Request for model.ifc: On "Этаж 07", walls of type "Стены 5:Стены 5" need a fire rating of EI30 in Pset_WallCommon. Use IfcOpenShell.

First a look at what the model holds.

```python
import ifcopenshell
import ifcopenshell.util.element

model = ifcopenshell.open("model.ifc")
print(model.schema)
storey = next(s for s in model.by_type("IfcBuildingStorey") if s.Name == "Этаж 07")
walls = [e for e in ifcopenshell.util.element.get_decomposition(storey) if e.is_a("IfcWall")]
seen = {}
for e in walls:
    element_type = ifcopenshell.util.element.get_type(e)
    key = (element_type.Name if element_type != e and element_type else None, ifcopenshell.util.element.get_pset(e, "Pset_WallCommon", "FireRating"))
    seen[key] = seen.get(key, 0) + 1
for (name, value), count in sorted(seen.items(), key=str):
    print(count, "x", name, "|", value)
```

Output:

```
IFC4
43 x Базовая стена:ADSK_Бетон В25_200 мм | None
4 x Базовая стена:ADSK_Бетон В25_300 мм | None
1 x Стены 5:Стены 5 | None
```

```python
import ifcopenshell
import ifcopenshell.api.pset
import ifcopenshell.util.element

model = ifcopenshell.open("model.ifc")

storey = next(s for s in model.by_type("IfcBuildingStorey") if s.Name == "Этаж 07")
walls = [e for e in ifcopenshell.util.element.get_decomposition(storey) if e.is_a("IfcWall")]

count = 0
for e in walls:
    element_type = ifcopenshell.util.element.get_type(e)
    if element_type in (None, e) or element_type.Name != "Стены 5:Стены 5":
        continue
    # add_pset returns the element's existing set when there is one.
    pset = ifcopenshell.api.pset.add_pset(model, product=e, name="Pset_WallCommon")
    ifcopenshell.api.pset.edit_pset(model, pset=pset, properties={"FireRating": "EI30"})
    count += 1

print(count, "walls updated")

model.write("model_rev.ifc")
```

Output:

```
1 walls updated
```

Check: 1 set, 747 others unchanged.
